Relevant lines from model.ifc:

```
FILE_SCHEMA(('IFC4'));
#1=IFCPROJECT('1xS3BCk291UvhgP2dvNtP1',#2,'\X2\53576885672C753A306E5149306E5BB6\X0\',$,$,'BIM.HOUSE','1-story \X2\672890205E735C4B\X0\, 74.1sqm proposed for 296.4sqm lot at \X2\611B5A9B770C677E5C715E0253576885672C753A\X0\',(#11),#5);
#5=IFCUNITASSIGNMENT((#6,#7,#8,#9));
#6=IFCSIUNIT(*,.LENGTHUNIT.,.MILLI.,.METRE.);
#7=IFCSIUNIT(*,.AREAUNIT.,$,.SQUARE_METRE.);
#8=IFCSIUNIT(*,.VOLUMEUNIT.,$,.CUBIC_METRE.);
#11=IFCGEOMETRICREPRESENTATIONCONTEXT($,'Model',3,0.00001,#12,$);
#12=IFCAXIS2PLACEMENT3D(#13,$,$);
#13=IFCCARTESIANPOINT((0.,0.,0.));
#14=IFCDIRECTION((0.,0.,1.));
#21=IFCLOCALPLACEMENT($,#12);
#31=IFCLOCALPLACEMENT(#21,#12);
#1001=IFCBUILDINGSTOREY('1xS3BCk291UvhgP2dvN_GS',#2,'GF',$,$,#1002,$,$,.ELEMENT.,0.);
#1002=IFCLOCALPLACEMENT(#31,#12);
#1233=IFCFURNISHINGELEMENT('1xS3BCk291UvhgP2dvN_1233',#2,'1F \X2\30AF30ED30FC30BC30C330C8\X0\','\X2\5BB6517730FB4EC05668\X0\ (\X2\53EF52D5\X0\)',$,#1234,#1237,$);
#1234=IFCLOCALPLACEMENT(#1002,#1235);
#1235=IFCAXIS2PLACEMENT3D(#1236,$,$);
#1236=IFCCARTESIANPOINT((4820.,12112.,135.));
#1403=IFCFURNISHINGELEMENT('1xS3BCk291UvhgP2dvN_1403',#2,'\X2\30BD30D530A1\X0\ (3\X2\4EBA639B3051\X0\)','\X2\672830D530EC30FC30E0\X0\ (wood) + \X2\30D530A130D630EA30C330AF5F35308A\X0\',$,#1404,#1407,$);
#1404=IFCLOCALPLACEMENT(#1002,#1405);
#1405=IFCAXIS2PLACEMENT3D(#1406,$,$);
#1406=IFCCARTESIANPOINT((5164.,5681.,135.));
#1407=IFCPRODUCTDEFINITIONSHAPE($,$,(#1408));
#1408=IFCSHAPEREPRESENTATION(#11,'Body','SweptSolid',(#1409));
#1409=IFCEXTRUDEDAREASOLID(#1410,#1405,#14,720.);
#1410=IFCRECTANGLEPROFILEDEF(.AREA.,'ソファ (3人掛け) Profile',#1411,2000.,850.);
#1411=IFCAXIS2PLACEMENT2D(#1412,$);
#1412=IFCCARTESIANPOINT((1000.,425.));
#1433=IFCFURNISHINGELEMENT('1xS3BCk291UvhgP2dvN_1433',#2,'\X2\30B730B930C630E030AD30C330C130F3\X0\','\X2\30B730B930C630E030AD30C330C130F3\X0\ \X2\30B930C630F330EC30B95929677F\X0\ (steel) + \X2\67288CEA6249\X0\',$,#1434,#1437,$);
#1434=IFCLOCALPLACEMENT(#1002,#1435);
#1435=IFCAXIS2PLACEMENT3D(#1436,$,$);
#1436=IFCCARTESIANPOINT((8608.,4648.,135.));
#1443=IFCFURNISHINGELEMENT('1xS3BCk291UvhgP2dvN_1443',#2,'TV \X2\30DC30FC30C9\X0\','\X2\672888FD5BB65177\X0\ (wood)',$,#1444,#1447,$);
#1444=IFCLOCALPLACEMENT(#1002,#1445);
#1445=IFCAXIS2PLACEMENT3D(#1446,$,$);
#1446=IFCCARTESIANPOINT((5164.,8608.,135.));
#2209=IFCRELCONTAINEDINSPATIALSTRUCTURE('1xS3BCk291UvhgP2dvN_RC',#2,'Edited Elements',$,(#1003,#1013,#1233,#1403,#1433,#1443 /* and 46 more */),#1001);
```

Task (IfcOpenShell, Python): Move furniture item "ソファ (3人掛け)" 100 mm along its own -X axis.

```python
import ifcopenshell
import ifcopenshell.api.geometry
import ifcopenshell.util.placement

model = ifcopenshell.open("model.ifc")

item = model.by_id(1403)
matrix = ifcopenshell.util.placement.get_local_placement(item.ObjectPlacement)
matrix[:3, 3] -= matrix[:3, 0] * 100.0
ifcopenshell.api.geometry.edit_object_placement(model, product=item, matrix=matrix, is_si=False)

print(ifcopenshell.util.placement.get_local_placement(item.ObjectPlacement).round(3) + 0.0)

model.write("model-out.ifc")
```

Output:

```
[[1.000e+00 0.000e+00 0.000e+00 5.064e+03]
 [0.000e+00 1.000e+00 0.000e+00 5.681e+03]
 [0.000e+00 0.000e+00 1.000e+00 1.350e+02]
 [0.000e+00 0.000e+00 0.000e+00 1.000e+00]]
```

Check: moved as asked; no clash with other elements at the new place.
